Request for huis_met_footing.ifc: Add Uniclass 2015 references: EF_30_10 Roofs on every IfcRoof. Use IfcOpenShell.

First a look at what the model holds.

```python
import ifcopenshell

model = ifcopenshell.open("huis_met_footing.ifc")
print(model.schema)
print("classifications:", [c.Name for c in model.by_type("IfcClassification")])
for ifc_class in ("IfcDoor", "IfcRoof", "IfcStair", "IfcWall", "IfcWindow"):
    print(ifc_class, len(model.by_type(ifc_class)))
```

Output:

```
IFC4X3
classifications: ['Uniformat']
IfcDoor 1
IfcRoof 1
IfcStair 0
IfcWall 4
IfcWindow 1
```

```python
import ifcopenshell
import ifcopenshell.api.classification

model = ifcopenshell.open("huis_met_footing.ifc")

system = ifcopenshell.api.classification.add_classification(model, classification="Uniclass 2015")

codes = {
    "IfcRoof": ("EF_30_10", "Roofs"),
}
for ifc_class, (code, name) in codes.items():
    products = model.by_type(ifc_class)
    ifcopenshell.api.classification.add_reference(
        model, products=products, classification=system, identification=code, name=name
    )
    print(code, len(products))

model.write("huis_met_footing_v2.ifc")
```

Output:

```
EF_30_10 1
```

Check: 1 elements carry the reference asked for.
